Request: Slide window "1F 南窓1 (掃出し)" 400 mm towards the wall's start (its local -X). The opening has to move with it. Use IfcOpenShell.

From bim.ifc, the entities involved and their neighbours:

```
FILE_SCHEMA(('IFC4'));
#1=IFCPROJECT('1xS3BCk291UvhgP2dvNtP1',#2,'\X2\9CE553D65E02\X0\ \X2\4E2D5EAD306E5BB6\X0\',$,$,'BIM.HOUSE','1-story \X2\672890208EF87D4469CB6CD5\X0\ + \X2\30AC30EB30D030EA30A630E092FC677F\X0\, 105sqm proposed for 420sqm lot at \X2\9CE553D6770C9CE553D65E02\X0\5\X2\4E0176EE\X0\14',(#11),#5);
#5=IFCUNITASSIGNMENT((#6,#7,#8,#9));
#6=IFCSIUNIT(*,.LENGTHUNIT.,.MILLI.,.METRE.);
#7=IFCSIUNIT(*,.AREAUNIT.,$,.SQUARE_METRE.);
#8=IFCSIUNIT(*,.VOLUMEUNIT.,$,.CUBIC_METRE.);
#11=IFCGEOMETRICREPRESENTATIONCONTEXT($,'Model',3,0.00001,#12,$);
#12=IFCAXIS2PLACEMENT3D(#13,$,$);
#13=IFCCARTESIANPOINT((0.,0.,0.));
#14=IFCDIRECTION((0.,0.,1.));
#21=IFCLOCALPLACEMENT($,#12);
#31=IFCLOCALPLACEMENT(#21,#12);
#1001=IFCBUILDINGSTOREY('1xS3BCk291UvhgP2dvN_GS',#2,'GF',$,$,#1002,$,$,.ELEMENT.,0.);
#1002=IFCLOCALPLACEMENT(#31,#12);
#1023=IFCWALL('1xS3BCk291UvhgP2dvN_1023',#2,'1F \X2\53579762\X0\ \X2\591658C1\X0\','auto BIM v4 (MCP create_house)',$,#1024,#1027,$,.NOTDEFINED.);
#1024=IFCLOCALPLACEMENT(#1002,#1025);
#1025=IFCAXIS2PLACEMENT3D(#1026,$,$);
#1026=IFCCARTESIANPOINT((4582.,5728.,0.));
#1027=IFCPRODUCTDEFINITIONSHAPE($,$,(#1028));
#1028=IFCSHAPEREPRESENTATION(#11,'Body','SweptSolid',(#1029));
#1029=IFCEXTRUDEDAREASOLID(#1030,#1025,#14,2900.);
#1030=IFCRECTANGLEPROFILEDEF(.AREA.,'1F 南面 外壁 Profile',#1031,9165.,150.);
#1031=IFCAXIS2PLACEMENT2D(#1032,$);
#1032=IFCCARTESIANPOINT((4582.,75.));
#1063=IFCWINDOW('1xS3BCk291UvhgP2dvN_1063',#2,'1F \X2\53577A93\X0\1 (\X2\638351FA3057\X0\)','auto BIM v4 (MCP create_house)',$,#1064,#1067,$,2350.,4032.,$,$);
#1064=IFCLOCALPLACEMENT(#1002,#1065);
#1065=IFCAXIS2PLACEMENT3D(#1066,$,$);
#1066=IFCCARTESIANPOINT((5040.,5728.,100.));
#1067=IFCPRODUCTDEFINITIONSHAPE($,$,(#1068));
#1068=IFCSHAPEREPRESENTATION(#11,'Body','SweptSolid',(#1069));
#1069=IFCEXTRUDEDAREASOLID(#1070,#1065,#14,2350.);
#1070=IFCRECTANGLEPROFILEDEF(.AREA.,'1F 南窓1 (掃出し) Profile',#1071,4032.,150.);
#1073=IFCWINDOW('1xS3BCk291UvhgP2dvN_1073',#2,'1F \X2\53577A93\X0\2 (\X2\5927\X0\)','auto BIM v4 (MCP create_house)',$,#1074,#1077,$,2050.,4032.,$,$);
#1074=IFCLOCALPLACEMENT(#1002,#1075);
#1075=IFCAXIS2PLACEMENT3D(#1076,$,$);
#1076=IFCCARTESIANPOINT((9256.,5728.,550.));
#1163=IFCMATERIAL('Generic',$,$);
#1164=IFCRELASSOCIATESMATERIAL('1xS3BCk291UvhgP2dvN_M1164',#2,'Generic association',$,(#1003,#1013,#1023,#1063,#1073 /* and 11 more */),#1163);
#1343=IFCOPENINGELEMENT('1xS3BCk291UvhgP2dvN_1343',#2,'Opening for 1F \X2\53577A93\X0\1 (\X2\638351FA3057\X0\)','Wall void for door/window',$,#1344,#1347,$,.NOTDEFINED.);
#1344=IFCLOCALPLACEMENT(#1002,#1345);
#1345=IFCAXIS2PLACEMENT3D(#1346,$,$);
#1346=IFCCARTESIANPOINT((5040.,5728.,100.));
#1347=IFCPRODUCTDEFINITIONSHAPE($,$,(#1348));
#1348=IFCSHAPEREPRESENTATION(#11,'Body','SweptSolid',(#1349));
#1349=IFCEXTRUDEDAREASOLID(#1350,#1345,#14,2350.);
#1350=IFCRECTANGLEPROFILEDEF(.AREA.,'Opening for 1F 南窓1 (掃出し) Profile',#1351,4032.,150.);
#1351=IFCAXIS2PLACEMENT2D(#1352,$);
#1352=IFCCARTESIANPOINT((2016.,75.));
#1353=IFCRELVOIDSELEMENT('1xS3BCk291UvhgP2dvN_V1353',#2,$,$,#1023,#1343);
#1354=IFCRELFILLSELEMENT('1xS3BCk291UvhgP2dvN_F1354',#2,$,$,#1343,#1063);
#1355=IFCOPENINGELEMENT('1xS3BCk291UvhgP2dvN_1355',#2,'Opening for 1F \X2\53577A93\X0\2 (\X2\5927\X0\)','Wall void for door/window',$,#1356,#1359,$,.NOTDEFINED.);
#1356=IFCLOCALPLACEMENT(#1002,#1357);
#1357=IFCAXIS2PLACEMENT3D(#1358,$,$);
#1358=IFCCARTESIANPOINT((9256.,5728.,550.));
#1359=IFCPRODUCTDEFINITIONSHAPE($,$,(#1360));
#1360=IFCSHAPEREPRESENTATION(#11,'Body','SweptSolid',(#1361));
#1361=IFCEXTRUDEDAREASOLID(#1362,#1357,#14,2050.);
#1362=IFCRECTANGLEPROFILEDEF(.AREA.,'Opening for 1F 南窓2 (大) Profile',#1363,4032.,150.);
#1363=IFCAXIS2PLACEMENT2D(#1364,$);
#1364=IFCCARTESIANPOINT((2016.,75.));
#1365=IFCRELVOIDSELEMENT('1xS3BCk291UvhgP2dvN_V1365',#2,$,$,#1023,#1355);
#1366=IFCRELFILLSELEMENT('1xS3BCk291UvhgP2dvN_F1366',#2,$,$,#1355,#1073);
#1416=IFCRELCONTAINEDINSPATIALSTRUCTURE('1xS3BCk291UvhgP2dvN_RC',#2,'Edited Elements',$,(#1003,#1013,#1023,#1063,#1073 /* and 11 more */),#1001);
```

```python
import ifcopenshell
import ifcopenshell.api.geometry
import ifcopenshell.util.placement

model = ifcopenshell.open("bim.ifc")

window = model.by_guid("1xS3BCk291UvhgP2dvN_1063")
opening = window.FillsVoids[0].RelatingOpeningElement
wall = opening.VoidsElements[0].RelatingBuildingElement

wall_matrix = ifcopenshell.util.placement.get_local_placement(wall.ObjectPlacement)
shift = wall_matrix[:3, 0] * -400.0
before = ifcopenshell.util.placement.get_local_placement(window.ObjectPlacement)[:3, 3].copy()

# The window is not placed relative to its opening, so move both.
for product in (opening, window):
    matrix = ifcopenshell.util.placement.get_local_placement(product.ObjectPlacement)
    matrix[:3, 3] += shift
    ifcopenshell.api.geometry.edit_object_placement(model, product=product, matrix=matrix, is_si=False)

after = ifcopenshell.util.placement.get_local_placement(window.ObjectPlacement)[:3, 3]
print("window moved by", (after - before).round(3) + 0.0)

model.write("bim_rev.ifc")
```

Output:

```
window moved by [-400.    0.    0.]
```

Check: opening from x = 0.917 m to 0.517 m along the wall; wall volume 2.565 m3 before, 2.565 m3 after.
